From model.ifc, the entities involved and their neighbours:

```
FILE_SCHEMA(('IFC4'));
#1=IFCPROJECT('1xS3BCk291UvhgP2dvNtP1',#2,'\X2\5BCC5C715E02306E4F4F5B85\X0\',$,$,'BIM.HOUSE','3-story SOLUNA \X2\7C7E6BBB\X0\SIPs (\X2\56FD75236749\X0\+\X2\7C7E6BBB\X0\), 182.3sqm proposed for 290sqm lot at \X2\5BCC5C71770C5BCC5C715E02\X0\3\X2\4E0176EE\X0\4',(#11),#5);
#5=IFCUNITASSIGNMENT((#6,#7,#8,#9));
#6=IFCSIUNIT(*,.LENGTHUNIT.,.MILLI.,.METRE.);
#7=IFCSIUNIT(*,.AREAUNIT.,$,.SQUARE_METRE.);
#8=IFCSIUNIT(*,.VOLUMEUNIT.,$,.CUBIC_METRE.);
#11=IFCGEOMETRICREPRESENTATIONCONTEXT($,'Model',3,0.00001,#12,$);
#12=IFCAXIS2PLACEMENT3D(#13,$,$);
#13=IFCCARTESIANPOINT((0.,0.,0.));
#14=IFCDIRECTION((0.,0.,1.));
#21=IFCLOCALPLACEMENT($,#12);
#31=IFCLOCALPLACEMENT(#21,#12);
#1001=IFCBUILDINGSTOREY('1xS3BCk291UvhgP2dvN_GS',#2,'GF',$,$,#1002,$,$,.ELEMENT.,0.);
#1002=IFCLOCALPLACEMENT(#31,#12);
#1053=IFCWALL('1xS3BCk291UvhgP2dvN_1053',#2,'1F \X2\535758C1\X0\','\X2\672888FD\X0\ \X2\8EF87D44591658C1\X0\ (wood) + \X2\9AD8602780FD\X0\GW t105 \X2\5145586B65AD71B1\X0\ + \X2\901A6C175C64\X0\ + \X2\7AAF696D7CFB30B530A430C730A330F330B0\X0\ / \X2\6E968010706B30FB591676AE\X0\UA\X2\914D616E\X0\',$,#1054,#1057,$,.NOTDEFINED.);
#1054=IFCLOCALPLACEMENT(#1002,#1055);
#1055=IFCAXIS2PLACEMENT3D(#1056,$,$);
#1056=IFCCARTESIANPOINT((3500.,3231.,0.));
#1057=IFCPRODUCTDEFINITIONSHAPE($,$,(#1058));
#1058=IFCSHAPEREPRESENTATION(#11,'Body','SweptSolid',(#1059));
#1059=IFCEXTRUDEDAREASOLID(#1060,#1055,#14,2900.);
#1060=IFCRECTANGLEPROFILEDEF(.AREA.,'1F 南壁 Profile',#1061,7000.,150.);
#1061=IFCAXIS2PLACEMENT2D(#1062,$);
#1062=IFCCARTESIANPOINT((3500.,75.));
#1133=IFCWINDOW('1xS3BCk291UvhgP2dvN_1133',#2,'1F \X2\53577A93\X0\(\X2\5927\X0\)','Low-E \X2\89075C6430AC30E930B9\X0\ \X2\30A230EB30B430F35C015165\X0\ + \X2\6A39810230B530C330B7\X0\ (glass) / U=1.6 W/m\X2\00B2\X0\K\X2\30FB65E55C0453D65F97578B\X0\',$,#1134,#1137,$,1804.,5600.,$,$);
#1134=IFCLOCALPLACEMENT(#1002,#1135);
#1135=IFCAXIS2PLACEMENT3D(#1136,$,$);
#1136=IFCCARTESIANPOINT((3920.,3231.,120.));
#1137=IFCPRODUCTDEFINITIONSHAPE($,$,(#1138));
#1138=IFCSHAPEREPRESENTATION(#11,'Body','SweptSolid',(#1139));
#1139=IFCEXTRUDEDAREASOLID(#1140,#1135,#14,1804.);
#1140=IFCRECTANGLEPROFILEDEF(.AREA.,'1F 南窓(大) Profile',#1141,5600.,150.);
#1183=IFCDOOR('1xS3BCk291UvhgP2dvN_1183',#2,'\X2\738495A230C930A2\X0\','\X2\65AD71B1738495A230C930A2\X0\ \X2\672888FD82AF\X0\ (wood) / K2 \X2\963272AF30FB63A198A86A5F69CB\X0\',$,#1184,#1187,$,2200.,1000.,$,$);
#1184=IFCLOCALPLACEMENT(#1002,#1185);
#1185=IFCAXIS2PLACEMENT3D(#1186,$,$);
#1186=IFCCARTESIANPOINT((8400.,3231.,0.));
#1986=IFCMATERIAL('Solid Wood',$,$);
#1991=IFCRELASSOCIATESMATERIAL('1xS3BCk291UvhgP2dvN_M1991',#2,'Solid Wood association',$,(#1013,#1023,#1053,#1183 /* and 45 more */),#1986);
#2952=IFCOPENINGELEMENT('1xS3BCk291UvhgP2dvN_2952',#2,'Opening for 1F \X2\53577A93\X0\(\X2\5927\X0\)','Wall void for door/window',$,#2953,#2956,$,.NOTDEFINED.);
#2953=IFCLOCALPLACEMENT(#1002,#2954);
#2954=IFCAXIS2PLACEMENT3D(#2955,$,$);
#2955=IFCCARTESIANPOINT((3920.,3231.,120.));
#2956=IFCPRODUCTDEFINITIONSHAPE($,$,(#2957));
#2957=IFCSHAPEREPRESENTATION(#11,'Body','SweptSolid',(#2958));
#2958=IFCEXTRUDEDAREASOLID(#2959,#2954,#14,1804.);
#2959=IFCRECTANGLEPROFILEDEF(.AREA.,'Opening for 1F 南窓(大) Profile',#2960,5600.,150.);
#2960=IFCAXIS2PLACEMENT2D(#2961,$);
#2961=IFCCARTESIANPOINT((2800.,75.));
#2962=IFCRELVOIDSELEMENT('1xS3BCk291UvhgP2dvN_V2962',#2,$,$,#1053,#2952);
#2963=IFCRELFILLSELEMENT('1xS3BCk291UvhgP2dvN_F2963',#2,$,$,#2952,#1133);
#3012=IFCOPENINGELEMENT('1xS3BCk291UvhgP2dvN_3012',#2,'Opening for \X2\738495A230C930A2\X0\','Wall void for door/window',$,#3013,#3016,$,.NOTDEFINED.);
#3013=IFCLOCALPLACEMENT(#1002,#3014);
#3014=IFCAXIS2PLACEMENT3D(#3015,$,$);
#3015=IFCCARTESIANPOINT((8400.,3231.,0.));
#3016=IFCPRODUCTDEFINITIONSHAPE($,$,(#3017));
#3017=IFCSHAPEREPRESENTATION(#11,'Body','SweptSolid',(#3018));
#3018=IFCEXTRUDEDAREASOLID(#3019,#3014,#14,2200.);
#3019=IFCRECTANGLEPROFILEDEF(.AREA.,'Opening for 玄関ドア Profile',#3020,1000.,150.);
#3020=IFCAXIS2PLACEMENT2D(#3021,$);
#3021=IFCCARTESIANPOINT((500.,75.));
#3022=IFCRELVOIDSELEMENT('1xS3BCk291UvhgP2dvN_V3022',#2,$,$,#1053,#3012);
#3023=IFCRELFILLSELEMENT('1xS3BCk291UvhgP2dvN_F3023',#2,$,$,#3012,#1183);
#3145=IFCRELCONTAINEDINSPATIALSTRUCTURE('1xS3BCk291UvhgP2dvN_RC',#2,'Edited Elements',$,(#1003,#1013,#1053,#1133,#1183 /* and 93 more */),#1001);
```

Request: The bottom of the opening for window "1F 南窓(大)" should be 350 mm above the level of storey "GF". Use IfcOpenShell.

```python
import numpy as np
import ifcopenshell
import ifcopenshell.api.geometry
import ifcopenshell.geom
import ifcopenshell.util.element
import ifcopenshell.util.placement
import ifcopenshell.util.shape
import ifcopenshell.util.unit

model = ifcopenshell.open("model.ifc")
unit_scale = ifcopenshell.util.unit.calculate_unit_scale(model)

window = model.by_guid("1xS3BCk291UvhgP2dvN_1133")
opening = window.FillsVoids[0].RelatingOpeningElement
storey = ifcopenshell.util.element.get_container(window, ifc_class="IfcBuildingStorey")
level = ifcopenshell.util.placement.get_local_placement(storey.ObjectPlacement)[2, 3]

# The opening's origin need not be at the sill, so measure its lowest point.
shape = ifcopenshell.geom.create_shape(ifcopenshell.geom.settings(), opening)
bottom = ifcopenshell.util.shape.get_shape_bottom_elevation(shape, shape.geometry) / unit_scale
dz = level + 0.35 / unit_scale - bottom

shift = np.array([0.0, 0.0, dz])
# The window is not placed relative to its opening, so move both.
for product in (opening, window):
    matrix = ifcopenshell.util.placement.get_local_placement(product.ObjectPlacement)
    matrix[:3, 3] += shift
    ifcopenshell.api.geometry.edit_object_placement(model, product=product, matrix=matrix, is_si=False)

print(f"moved by {dz * unit_scale:+.3f} m")

model.write("model_v2.ifc")
```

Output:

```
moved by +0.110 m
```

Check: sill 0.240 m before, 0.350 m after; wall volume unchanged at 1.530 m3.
